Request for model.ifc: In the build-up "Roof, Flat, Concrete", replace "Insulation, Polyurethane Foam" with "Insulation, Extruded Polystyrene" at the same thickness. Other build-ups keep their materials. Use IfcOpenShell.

First a look at what the model holds.

```python
import ifcopenshell
import ifcopenshell.util.element

model = ifcopenshell.open("model.ifc")
print(model.schema)
for layer_set in model.by_type("IfcMaterialLayerSet"):
    if layer_set.LayerSetName == "Roof, Flat, Concrete":
        for layer in layer_set.MaterialLayers:
            print(layer.id(), layer.Material and layer.Material.Name, layer.LayerThickness, sep=" | ")
        print(len(ifcopenshell.util.element.get_elements_by_material(model, layer_set)), "elements and types use it")
print(sorted(m.Name for m in model.by_type("IfcMaterial") if m.Name)[:60])
```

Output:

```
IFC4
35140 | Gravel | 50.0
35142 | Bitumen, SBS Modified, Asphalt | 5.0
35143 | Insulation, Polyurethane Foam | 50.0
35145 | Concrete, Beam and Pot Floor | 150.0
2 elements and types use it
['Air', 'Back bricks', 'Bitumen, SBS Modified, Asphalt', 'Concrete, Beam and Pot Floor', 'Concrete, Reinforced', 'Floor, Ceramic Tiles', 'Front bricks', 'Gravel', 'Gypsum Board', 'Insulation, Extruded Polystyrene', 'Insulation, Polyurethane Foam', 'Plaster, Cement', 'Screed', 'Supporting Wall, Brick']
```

```python
import ifcopenshell
import ifcopenshell.api.material

model = ifcopenshell.open("model.ifc")

layer_set = next(s for s in model.by_type("IfcMaterialLayerSet") if s.LayerSetName == "Roof, Flat, Concrete")
layer = next(l for l in layer_set.MaterialLayers if l.Material and l.Material.Name == "Insulation, Polyurethane Foam")
material = next(m for m in model.by_type("IfcMaterial") if m.Name == "Insulation, Extruded Polystyrene")

# Point this one layer at the other material; renaming the old one would change it everywhere.
ifcopenshell.api.material.edit_layer(model, layer=layer, attributes={}, material=material)

print([l.Material.Name if l.Material else None for l in layer_set.MaterialLayers])

model.write("model-out.ifc")
```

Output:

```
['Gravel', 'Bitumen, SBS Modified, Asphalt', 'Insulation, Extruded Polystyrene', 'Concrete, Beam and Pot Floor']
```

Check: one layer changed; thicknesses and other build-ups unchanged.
